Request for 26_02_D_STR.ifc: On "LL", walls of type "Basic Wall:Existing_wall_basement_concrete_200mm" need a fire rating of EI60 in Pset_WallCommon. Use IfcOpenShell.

First a look at what the model holds.

```python
import ifcopenshell
import ifcopenshell.util.element

model = ifcopenshell.open("26_02_D_STR.ifc")
print(model.schema)
storey = next(s for s in model.by_type("IfcBuildingStorey") if s.Name == "LL")
walls = [e for e in ifcopenshell.util.element.get_decomposition(storey) if e.is_a("IfcWall")]
seen = {}
for e in walls:
    element_type = ifcopenshell.util.element.get_type(e)
    key = (element_type.Name if element_type != e and element_type else None, ifcopenshell.util.element.get_pset(e, "Pset_WallCommon", "FireRating"))
    seen[key] = seen.get(key, 0) + 1
for (name, value), count in sorted(seen.items(), key=str):
    print(count, "x", name, "|", value)
```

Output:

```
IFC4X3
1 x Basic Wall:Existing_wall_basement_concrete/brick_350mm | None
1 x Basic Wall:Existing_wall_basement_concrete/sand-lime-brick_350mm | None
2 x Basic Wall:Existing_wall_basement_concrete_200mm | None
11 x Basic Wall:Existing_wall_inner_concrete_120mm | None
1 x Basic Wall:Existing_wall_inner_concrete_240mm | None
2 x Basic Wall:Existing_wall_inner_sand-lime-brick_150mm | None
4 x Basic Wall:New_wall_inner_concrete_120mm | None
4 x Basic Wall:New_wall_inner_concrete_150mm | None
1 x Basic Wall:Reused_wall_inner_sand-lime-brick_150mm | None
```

```python
import ifcopenshell
import ifcopenshell.api.pset
import ifcopenshell.util.element

model = ifcopenshell.open("26_02_D_STR.ifc")

storey = next(s for s in model.by_type("IfcBuildingStorey") if s.Name == "LL")
walls = [e for e in ifcopenshell.util.element.get_decomposition(storey) if e.is_a("IfcWall")]

count = 0
for e in walls:
    element_type = ifcopenshell.util.element.get_type(e)
    if element_type in (None, e) or element_type.Name != "Basic Wall:Existing_wall_basement_concrete_200mm":
        continue
    # add_pset returns the element's existing set when there is one.
    pset = ifcopenshell.api.pset.add_pset(model, product=e, name="Pset_WallCommon")
    ifcopenshell.api.pset.edit_pset(model, pset=pset, properties={"FireRating": "EI60"})
    count += 1

print(count, "walls updated")

model.write("26_02_D_STR-out.ifc")
```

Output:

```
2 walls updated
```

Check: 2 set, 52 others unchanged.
